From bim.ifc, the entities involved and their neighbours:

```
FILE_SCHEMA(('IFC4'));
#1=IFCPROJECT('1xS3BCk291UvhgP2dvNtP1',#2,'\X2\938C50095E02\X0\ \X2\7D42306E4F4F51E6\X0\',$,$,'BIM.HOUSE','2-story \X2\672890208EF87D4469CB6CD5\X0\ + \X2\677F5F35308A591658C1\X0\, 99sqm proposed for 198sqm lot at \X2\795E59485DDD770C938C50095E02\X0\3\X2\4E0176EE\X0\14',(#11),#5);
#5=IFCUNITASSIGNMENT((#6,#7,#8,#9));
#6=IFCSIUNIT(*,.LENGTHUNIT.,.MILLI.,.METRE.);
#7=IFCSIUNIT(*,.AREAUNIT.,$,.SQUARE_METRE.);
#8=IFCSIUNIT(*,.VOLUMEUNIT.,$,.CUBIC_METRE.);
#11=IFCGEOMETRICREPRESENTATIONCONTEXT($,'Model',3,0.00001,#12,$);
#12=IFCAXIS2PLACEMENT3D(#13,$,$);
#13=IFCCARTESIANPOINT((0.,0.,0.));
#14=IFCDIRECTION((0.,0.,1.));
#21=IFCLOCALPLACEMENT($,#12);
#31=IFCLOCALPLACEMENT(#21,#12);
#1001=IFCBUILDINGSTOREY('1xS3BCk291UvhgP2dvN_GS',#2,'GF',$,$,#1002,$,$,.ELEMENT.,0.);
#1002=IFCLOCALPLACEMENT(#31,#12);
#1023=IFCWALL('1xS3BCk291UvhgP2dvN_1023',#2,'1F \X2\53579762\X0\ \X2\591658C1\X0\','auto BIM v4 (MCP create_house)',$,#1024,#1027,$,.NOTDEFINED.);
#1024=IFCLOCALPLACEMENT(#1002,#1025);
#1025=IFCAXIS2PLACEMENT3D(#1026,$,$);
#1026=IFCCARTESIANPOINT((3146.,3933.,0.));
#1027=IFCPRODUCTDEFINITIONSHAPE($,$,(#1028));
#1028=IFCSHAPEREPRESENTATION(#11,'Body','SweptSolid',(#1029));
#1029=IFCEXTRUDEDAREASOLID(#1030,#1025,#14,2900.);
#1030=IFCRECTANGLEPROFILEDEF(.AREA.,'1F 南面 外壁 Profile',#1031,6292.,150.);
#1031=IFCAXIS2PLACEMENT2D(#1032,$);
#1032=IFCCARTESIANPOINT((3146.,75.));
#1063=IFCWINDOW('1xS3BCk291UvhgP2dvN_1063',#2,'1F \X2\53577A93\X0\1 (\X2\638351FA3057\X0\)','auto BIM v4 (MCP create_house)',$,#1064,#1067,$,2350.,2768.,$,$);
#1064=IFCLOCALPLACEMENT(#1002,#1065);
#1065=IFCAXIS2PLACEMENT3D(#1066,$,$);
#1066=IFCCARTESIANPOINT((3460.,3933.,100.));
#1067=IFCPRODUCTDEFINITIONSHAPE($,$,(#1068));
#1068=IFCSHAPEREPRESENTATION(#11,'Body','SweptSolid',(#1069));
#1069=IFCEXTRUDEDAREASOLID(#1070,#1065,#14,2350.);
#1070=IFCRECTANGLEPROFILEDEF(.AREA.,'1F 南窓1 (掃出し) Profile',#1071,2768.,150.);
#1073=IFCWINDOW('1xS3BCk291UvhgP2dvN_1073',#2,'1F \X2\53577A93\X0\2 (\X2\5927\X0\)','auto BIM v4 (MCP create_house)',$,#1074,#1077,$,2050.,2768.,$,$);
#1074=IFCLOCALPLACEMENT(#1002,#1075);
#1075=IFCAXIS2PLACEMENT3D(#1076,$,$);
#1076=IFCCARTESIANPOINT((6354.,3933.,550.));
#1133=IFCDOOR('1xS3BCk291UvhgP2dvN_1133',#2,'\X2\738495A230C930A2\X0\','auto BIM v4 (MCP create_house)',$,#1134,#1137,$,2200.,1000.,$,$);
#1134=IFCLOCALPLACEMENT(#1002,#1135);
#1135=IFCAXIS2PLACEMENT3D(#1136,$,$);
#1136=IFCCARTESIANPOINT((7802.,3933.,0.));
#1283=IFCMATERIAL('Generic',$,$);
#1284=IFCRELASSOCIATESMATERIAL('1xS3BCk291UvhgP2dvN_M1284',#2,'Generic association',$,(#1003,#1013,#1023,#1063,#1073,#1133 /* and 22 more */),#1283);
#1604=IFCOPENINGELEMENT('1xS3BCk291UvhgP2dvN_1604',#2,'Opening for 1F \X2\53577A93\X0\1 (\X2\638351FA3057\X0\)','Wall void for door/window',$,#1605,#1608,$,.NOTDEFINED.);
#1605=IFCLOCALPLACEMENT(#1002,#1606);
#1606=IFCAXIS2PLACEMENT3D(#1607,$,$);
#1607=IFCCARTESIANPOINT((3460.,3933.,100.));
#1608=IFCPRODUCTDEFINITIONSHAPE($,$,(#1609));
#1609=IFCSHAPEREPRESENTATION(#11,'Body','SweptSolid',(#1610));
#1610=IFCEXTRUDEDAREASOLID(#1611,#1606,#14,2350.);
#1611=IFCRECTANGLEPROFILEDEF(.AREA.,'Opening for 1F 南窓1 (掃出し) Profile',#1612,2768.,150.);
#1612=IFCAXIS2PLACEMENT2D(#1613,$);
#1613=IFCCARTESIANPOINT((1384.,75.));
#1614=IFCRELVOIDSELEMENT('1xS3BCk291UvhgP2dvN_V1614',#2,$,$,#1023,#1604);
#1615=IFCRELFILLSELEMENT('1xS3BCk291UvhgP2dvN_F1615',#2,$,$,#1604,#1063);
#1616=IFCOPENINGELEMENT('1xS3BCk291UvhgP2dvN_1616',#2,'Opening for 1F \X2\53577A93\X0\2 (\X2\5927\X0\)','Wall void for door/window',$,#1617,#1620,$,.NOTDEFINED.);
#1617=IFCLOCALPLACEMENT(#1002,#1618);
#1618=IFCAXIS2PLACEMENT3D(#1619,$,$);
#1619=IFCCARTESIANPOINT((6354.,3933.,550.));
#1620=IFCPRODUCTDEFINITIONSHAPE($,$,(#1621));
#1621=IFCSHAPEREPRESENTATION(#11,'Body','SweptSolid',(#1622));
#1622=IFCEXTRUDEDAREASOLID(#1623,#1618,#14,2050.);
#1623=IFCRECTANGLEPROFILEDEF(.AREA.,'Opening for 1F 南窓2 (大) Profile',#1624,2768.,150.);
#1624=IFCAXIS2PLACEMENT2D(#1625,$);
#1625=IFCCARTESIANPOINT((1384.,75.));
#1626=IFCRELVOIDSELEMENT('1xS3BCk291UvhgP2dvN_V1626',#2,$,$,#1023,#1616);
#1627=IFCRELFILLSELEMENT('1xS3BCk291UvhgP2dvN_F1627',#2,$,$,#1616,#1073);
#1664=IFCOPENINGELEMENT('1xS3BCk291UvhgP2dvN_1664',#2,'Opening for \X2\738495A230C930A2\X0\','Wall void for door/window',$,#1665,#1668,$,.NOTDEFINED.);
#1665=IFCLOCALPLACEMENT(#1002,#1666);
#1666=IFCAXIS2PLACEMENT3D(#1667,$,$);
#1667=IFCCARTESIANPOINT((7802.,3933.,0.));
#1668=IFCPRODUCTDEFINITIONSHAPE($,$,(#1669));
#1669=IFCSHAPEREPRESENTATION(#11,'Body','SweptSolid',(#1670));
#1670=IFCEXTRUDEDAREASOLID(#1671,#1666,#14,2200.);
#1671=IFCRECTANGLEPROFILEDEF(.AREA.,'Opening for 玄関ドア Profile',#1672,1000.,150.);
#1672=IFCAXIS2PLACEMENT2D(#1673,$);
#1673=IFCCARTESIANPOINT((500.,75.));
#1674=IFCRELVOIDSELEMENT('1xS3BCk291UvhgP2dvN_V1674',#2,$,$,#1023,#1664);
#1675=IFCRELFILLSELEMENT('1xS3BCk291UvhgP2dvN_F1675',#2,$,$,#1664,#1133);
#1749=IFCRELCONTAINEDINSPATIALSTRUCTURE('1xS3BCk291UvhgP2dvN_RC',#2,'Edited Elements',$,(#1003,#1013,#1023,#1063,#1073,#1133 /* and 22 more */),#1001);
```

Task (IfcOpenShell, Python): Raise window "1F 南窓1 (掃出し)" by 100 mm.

```python
import numpy as np
import ifcopenshell
import ifcopenshell.api.geometry
import ifcopenshell.util.placement
import ifcopenshell.util.unit

model = ifcopenshell.open("bim.ifc")
unit_scale = ifcopenshell.util.unit.calculate_unit_scale(model)

window = model.by_guid("1xS3BCk291UvhgP2dvN_1063")
opening = window.FillsVoids[0].RelatingOpeningElement
dz = 100.0

shift = np.array([0.0, 0.0, dz])
# The window is not placed relative to its opening, so move both.
for product in (opening, window):
    matrix = ifcopenshell.util.placement.get_local_placement(product.ObjectPlacement)
    matrix[:3, 3] += shift
    ifcopenshell.api.geometry.edit_object_placement(model, product=product, matrix=matrix, is_si=False)

print(f"moved by {dz * unit_scale:+.3f} m")

model.write("bim_rev.ifc")
```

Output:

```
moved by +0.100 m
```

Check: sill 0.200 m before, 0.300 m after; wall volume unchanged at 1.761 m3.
